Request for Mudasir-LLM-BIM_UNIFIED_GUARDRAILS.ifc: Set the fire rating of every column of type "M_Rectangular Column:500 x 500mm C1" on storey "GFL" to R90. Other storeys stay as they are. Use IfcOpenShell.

First a look at what the model holds.

```python
import ifcopenshell
import ifcopenshell.util.element

model = ifcopenshell.open("Mudasir-LLM-BIM_UNIFIED_GUARDRAILS.ifc")
print(model.schema)
storey = next(s for s in model.by_type("IfcBuildingStorey") if s.Name == "GFL")
columns = [e for e in ifcopenshell.util.element.get_decomposition(storey) if e.is_a("IfcColumn")]
seen = {}
for e in columns:
    element_type = ifcopenshell.util.element.get_type(e)
    key = (element_type.Name if element_type != e and element_type else None, ifcopenshell.util.element.get_pset(e, "Pset_ColumnCommon", "FireRating"))
    seen[key] = seen.get(key, 0) + 1
for (name, value), count in sorted(seen.items(), key=str):
    print(count, "x", name, "|", value)
```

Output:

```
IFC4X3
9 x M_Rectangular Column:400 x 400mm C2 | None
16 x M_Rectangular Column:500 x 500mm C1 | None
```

```python
import ifcopenshell
import ifcopenshell.api.pset
import ifcopenshell.util.element

model = ifcopenshell.open("Mudasir-LLM-BIM_UNIFIED_GUARDRAILS.ifc")

storey = next(s for s in model.by_type("IfcBuildingStorey") if s.Name == "GFL")
columns = [e for e in ifcopenshell.util.element.get_decomposition(storey) if e.is_a("IfcColumn")]

count = 0
for e in columns:
    element_type = ifcopenshell.util.element.get_type(e)
    if element_type in (None, e) or element_type.Name != "M_Rectangular Column:500 x 500mm C1":
        continue
    # add_pset returns the element's existing set when there is one.
    pset = ifcopenshell.api.pset.add_pset(model, product=e, name="Pset_ColumnCommon")
    ifcopenshell.api.pset.edit_pset(model, pset=pset, properties={"FireRating": "R90"})
    count += 1

print(count, "columns updated")

model.write("Mudasir-LLM-BIM_UNIFIED_GUARDRAILS_edited.ifc")
```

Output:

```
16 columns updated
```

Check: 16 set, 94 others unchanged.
